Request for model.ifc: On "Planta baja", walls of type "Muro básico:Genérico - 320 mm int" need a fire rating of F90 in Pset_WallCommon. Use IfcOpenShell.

First a look at what the model holds.

```python
import ifcopenshell
import ifcopenshell.util.element

model = ifcopenshell.open("model.ifc")
print(model.schema)
storey = next(s for s in model.by_type("IfcBuildingStorey") if s.Name == "Planta baja")
walls = [e for e in ifcopenshell.util.element.get_decomposition(storey) if e.is_a("IfcWall")]
seen = {}
for e in walls:
    element_type = ifcopenshell.util.element.get_type(e)
    key = (element_type.Name if element_type != e and element_type else None, ifcopenshell.util.element.get_pset(e, "Pset_WallCommon", "FireRating"))
    seen[key] = seen.get(key, 0) + 1
for (name, value), count in sorted(seen.items(), key=str):
    print(count, "x", name, "|", value)
```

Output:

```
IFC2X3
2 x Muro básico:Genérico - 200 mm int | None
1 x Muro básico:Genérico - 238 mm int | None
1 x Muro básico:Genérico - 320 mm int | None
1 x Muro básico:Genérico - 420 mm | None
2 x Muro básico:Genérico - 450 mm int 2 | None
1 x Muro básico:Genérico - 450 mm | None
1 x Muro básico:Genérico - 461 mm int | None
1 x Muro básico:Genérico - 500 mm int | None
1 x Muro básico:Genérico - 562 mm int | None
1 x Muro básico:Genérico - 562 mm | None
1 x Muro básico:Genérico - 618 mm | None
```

```python
import ifcopenshell
import ifcopenshell.api.pset
import ifcopenshell.util.element

model = ifcopenshell.open("model.ifc")

storey = next(s for s in model.by_type("IfcBuildingStorey") if s.Name == "Planta baja")
walls = [e for e in ifcopenshell.util.element.get_decomposition(storey) if e.is_a("IfcWall")]

count = 0
for e in walls:
    element_type = ifcopenshell.util.element.get_type(e)
    if element_type in (None, e) or element_type.Name != "Muro básico:Genérico - 320 mm int":
        continue
    # add_pset returns the element's existing set when there is one.
    pset = ifcopenshell.api.pset.add_pset(model, product=e, name="Pset_WallCommon")
    ifcopenshell.api.pset.edit_pset(model, pset=pset, properties={"FireRating": "F90"})
    count += 1

print(count, "walls updated")

model.write("model_updated.ifc")
```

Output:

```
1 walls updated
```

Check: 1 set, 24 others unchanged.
